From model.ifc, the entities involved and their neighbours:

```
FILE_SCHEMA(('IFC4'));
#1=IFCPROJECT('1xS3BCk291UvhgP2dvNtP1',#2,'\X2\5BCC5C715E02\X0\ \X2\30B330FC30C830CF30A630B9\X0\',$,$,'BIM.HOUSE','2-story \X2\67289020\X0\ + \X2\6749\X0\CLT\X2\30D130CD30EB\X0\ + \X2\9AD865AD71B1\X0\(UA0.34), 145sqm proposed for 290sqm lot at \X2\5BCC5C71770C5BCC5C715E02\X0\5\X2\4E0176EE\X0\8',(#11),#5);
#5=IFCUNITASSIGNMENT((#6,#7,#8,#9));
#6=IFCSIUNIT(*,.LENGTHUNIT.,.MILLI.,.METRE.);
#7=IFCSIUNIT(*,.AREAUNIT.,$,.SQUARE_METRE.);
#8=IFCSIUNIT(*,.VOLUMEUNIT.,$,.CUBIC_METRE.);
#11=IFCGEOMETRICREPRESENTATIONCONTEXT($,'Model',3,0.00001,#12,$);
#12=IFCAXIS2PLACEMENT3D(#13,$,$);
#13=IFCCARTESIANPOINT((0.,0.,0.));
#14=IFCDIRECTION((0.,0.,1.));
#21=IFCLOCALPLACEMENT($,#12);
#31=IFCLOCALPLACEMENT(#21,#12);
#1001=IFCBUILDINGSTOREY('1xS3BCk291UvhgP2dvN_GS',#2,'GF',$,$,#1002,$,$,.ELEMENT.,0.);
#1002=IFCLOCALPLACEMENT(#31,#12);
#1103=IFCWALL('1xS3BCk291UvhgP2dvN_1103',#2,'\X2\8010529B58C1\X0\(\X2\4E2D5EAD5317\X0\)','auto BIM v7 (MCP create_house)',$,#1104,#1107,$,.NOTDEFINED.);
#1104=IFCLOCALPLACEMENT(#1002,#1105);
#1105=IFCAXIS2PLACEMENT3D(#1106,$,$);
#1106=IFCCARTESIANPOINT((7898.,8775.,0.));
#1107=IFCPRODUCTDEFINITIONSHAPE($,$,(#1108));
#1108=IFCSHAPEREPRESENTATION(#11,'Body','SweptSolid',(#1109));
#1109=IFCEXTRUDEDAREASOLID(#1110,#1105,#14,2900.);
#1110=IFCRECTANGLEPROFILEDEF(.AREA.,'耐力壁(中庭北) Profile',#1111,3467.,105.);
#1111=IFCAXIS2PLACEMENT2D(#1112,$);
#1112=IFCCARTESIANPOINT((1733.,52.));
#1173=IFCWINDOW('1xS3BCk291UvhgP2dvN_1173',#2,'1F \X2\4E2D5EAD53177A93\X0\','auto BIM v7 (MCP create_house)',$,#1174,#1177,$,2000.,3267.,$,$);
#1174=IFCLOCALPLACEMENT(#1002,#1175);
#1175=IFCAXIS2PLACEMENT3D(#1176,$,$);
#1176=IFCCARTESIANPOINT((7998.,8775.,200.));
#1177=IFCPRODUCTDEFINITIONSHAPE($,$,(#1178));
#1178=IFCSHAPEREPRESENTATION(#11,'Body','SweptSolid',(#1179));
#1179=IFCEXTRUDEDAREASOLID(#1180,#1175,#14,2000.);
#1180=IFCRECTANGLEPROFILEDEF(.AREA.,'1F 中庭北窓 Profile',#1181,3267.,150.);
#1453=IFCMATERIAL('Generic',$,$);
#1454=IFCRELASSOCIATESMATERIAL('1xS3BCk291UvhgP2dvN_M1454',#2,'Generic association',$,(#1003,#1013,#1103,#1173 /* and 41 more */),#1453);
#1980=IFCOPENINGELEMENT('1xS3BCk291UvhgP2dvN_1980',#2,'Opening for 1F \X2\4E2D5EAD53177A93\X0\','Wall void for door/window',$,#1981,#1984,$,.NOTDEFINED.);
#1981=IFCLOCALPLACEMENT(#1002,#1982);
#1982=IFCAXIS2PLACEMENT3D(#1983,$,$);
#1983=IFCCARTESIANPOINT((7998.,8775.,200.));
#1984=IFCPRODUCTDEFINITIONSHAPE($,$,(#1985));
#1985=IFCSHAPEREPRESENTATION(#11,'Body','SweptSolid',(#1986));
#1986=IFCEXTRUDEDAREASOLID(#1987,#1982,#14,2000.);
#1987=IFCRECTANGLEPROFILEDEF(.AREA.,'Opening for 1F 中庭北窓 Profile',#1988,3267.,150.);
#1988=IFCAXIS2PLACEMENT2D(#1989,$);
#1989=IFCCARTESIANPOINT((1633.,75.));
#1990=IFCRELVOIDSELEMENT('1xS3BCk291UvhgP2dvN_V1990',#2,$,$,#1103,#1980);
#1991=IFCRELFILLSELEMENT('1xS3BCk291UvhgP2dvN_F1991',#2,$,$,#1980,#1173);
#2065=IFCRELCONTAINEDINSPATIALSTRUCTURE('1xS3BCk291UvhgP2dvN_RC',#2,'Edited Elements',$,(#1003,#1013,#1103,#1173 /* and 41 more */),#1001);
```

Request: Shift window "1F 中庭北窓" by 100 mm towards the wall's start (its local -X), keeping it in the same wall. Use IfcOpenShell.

```python
import ifcopenshell
import ifcopenshell.api.geometry
import ifcopenshell.util.placement
import ifcopenshell.util.unit

model = ifcopenshell.open("model.ifc")
unit_scale = ifcopenshell.util.unit.calculate_unit_scale(model)

window = model.by_guid("1xS3BCk291UvhgP2dvN_1173")
opening = window.FillsVoids[0].RelatingOpeningElement
wall = opening.VoidsElements[0].RelatingBuildingElement

wall_matrix = ifcopenshell.util.placement.get_local_placement(wall.ObjectPlacement)
shift = wall_matrix[:3, 0] * -0.1 / unit_scale
before = ifcopenshell.util.placement.get_local_placement(window.ObjectPlacement)[:3, 3].copy()

# The window is not placed relative to its opening, so move both.
for product in (opening, window):
    matrix = ifcopenshell.util.placement.get_local_placement(product.ObjectPlacement)
    matrix[:3, 3] += shift
    ifcopenshell.api.geometry.edit_object_placement(model, product=product, matrix=matrix, is_si=False)

after = ifcopenshell.util.placement.get_local_placement(window.ObjectPlacement)[:3, 3]
print("window moved by", (after - before).round(3) + 0.0)

model.write("model_edited.ifc")
```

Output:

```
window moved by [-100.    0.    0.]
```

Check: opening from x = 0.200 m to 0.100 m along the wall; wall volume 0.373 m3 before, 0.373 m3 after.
